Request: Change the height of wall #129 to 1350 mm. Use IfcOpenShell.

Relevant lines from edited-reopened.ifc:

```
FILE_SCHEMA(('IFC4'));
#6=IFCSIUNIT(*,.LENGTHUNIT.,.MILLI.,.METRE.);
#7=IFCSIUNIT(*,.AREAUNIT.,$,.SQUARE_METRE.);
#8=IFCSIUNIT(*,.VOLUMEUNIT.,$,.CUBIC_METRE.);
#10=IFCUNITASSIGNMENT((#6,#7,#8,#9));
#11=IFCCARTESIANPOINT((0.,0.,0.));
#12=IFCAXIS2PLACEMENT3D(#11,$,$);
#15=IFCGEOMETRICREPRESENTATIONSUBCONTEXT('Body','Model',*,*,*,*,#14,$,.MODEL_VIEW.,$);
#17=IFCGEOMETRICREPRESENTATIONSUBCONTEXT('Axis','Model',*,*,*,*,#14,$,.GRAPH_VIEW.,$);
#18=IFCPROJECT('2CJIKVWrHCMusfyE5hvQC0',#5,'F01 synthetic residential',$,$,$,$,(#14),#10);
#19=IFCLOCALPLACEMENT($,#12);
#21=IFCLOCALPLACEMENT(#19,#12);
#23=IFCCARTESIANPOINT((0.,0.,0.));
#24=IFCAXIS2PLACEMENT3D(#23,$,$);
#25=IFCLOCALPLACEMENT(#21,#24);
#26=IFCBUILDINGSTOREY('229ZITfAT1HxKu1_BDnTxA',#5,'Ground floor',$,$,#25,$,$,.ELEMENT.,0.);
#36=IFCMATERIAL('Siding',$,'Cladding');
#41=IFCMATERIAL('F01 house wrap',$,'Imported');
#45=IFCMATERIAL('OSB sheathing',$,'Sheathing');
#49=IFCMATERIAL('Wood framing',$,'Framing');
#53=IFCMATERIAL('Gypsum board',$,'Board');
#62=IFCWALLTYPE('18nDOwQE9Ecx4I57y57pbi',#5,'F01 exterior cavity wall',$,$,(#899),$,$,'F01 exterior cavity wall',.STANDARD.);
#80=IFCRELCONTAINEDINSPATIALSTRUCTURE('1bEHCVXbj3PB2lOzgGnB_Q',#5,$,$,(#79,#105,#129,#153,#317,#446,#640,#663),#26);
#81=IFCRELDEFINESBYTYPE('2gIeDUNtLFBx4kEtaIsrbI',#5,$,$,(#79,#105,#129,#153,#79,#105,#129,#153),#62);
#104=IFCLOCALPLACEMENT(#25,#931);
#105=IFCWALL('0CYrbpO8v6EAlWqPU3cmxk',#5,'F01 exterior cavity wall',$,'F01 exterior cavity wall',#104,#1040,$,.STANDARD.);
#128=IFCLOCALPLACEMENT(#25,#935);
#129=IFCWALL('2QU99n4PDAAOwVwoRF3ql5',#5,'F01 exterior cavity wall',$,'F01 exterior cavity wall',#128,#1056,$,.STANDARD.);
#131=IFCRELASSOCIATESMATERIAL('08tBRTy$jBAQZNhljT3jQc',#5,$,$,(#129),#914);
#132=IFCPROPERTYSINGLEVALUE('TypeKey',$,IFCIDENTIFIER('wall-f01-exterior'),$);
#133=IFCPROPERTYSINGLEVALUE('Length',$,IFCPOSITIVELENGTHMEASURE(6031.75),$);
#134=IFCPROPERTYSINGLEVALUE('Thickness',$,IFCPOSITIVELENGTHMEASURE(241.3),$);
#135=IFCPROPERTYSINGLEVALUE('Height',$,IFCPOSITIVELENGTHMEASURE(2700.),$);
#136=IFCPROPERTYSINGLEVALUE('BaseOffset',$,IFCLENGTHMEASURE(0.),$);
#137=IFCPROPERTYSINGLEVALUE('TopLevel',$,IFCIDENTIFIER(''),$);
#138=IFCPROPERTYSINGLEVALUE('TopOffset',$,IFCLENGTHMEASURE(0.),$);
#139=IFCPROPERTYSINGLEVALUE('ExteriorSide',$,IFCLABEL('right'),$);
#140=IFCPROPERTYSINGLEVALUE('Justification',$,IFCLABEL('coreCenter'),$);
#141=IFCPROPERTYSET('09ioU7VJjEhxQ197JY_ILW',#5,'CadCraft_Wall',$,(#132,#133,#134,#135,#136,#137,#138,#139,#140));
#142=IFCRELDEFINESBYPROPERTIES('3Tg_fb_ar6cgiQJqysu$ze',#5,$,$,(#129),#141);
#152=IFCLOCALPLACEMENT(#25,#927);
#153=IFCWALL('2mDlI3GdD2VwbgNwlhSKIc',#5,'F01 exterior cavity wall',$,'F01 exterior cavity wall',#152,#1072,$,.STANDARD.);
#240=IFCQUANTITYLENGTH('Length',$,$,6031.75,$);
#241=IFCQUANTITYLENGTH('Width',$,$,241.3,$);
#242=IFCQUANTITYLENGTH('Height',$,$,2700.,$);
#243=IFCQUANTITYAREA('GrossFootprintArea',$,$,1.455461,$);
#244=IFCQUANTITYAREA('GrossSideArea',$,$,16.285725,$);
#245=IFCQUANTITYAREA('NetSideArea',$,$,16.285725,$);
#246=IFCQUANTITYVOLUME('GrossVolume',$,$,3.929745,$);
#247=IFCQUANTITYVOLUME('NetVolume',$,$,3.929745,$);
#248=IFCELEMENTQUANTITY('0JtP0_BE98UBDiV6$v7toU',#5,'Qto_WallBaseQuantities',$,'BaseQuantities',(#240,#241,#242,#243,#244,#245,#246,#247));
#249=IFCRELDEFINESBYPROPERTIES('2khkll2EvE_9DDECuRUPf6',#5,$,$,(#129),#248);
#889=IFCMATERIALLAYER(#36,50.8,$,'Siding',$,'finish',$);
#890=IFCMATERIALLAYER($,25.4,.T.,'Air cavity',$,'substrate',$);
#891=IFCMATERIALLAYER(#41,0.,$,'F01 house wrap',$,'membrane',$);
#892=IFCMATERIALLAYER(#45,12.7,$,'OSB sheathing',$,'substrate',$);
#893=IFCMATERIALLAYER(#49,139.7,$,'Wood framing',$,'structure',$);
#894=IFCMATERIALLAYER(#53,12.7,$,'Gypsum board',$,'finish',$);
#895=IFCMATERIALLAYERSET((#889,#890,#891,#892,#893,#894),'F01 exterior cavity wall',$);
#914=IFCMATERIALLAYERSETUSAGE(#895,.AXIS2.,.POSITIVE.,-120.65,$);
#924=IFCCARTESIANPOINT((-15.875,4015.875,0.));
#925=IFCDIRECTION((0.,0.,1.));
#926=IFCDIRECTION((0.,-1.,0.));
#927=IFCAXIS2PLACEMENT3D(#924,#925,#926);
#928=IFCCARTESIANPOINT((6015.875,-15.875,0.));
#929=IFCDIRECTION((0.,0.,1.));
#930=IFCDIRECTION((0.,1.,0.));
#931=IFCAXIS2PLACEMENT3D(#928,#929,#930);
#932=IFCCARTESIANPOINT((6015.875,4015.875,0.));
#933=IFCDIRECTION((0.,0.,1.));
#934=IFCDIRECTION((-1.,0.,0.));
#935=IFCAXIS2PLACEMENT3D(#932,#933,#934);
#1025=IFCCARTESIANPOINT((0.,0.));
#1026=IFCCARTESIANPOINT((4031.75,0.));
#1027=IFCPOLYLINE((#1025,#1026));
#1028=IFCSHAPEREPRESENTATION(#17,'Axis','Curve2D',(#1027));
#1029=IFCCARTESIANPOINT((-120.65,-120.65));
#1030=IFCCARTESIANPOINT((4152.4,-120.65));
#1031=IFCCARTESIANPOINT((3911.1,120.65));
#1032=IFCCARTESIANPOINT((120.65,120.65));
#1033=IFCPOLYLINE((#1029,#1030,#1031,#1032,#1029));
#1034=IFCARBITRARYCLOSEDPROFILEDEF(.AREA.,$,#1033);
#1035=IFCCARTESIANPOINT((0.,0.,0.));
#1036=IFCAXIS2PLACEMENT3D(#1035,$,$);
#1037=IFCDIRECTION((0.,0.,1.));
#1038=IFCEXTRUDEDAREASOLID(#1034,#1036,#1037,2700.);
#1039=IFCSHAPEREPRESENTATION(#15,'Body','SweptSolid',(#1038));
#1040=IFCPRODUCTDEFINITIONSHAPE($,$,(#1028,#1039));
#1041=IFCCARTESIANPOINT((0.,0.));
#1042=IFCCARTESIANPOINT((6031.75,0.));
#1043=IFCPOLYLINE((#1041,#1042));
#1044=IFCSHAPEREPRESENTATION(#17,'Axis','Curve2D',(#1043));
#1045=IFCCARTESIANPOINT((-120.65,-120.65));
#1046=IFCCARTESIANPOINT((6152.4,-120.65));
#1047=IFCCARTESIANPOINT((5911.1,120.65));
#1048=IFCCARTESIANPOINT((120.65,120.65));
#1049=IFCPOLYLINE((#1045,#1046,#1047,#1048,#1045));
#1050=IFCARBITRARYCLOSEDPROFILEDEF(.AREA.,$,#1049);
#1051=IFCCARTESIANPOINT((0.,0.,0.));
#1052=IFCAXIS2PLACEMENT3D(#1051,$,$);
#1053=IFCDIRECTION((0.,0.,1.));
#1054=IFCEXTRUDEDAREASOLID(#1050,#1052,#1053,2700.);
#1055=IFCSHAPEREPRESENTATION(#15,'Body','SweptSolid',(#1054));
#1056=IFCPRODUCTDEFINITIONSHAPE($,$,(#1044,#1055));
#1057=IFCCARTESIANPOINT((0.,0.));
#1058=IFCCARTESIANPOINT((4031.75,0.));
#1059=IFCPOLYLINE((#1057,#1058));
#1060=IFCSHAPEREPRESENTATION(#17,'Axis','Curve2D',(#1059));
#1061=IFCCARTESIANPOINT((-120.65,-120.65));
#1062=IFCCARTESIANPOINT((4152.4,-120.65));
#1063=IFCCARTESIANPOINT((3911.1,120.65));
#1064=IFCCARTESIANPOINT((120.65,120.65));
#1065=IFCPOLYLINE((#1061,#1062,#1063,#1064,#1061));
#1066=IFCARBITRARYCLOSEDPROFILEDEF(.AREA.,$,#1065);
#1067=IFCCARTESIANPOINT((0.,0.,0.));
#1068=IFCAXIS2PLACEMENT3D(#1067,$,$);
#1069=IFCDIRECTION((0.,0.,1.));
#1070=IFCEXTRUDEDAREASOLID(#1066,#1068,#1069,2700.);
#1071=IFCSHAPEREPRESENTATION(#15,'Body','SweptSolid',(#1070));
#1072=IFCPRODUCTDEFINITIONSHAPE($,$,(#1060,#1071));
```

```python
import ifcopenshell
import ifcopenshell.api.pset
import ifcopenshell.geom
import ifcopenshell.util.element
import ifcopenshell.util.representation
import ifcopenshell.util.shape
import ifcopenshell.util.unit

model = ifcopenshell.open("edited-reopened.ifc")
unit_scale = ifcopenshell.util.unit.calculate_unit_scale(model)
area_scale = ifcopenshell.util.unit.calculate_unit_scale(model, "AREAUNIT")
volume_scale = ifcopenshell.util.unit.calculate_unit_scale(model, "VOLUMEUNIT")
settings = ifcopenshell.geom.settings()


def volume(element):
    """Net volume in cubic metres, openings subtracted."""
    shape = ifcopenshell.geom.create_shape(settings, element)
    return ifcopenshell.util.shape.get_volume(shape.geometry)


wall = model.by_id(129)
before = volume(wall)

body = ifcopenshell.util.representation.get_representation(wall, "Model", "Body")
solid = body.Items[0]
old_height = solid.Depth
solid.Depth = 1.35 / unit_scale
after = volume(wall)
thickness = 0.2413  # wall thickness in metres

# Update the stored height, areas and volumes.
pset = model.by_id(ifcopenshell.util.element.get_pset(wall, "CadCraft_Wall", should_inherit=False)["id"])
ifcopenshell.api.pset.edit_pset(model, pset=pset, properties={
    "Height": model.create_entity("IfcPositiveLengthMeasure", solid.Depth),
})
qto = model.by_id(ifcopenshell.util.element.get_pset(wall, "Qto_WallBaseQuantities", should_inherit=False)["id"])
ifcopenshell.api.pset.edit_qto(model, qto=qto, properties={
    "Height": solid.Depth,
    "GrossSideArea": ifcopenshell.util.element.get_pset(wall, "Qto_WallBaseQuantities", "GrossSideArea") * solid.Depth / old_height,
    "NetSideArea": after / thickness / area_scale,
    "GrossVolume": ifcopenshell.util.element.get_pset(wall, "Qto_WallBaseQuantities", "GrossVolume") * solid.Depth / old_height,
    "NetVolume": after / volume_scale,
})

print(f"height {old_height:g} -> {solid.Depth:g}, volume {before:.3f} -> {after:.3f} m3")

model.write("edited-reopened_rev.ifc")
```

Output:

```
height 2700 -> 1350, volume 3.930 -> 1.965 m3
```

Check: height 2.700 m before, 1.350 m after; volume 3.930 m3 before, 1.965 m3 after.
